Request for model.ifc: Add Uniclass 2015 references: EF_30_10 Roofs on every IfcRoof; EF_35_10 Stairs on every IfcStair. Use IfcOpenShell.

First a look at what the model holds.

```python
import ifcopenshell

model = ifcopenshell.open("model.ifc")
print(model.schema)
print("classifications:", [c.Name for c in model.by_type("IfcClassification")])
for ifc_class in ("IfcDoor", "IfcRoof", "IfcStair", "IfcWall", "IfcWindow"):
    print(ifc_class, len(model.by_type(ifc_class)))
```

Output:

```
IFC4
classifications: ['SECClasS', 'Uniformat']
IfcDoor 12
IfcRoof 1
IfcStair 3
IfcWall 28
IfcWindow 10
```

```python
import ifcopenshell
import ifcopenshell.api.classification

model = ifcopenshell.open("model.ifc")

system = ifcopenshell.api.classification.add_classification(model, classification="Uniclass 2015")

codes = {
    "IfcRoof": ("EF_30_10", "Roofs"),
    "IfcStair": ("EF_35_10", "Stairs"),
}
for ifc_class, (code, name) in codes.items():
    products = model.by_type(ifc_class)
    ifcopenshell.api.classification.add_reference(
        model, products=products, classification=system, identification=code, name=name
    )
    print(code, len(products))

model.write("model_v2.ifc")
```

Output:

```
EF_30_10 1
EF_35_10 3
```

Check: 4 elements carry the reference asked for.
